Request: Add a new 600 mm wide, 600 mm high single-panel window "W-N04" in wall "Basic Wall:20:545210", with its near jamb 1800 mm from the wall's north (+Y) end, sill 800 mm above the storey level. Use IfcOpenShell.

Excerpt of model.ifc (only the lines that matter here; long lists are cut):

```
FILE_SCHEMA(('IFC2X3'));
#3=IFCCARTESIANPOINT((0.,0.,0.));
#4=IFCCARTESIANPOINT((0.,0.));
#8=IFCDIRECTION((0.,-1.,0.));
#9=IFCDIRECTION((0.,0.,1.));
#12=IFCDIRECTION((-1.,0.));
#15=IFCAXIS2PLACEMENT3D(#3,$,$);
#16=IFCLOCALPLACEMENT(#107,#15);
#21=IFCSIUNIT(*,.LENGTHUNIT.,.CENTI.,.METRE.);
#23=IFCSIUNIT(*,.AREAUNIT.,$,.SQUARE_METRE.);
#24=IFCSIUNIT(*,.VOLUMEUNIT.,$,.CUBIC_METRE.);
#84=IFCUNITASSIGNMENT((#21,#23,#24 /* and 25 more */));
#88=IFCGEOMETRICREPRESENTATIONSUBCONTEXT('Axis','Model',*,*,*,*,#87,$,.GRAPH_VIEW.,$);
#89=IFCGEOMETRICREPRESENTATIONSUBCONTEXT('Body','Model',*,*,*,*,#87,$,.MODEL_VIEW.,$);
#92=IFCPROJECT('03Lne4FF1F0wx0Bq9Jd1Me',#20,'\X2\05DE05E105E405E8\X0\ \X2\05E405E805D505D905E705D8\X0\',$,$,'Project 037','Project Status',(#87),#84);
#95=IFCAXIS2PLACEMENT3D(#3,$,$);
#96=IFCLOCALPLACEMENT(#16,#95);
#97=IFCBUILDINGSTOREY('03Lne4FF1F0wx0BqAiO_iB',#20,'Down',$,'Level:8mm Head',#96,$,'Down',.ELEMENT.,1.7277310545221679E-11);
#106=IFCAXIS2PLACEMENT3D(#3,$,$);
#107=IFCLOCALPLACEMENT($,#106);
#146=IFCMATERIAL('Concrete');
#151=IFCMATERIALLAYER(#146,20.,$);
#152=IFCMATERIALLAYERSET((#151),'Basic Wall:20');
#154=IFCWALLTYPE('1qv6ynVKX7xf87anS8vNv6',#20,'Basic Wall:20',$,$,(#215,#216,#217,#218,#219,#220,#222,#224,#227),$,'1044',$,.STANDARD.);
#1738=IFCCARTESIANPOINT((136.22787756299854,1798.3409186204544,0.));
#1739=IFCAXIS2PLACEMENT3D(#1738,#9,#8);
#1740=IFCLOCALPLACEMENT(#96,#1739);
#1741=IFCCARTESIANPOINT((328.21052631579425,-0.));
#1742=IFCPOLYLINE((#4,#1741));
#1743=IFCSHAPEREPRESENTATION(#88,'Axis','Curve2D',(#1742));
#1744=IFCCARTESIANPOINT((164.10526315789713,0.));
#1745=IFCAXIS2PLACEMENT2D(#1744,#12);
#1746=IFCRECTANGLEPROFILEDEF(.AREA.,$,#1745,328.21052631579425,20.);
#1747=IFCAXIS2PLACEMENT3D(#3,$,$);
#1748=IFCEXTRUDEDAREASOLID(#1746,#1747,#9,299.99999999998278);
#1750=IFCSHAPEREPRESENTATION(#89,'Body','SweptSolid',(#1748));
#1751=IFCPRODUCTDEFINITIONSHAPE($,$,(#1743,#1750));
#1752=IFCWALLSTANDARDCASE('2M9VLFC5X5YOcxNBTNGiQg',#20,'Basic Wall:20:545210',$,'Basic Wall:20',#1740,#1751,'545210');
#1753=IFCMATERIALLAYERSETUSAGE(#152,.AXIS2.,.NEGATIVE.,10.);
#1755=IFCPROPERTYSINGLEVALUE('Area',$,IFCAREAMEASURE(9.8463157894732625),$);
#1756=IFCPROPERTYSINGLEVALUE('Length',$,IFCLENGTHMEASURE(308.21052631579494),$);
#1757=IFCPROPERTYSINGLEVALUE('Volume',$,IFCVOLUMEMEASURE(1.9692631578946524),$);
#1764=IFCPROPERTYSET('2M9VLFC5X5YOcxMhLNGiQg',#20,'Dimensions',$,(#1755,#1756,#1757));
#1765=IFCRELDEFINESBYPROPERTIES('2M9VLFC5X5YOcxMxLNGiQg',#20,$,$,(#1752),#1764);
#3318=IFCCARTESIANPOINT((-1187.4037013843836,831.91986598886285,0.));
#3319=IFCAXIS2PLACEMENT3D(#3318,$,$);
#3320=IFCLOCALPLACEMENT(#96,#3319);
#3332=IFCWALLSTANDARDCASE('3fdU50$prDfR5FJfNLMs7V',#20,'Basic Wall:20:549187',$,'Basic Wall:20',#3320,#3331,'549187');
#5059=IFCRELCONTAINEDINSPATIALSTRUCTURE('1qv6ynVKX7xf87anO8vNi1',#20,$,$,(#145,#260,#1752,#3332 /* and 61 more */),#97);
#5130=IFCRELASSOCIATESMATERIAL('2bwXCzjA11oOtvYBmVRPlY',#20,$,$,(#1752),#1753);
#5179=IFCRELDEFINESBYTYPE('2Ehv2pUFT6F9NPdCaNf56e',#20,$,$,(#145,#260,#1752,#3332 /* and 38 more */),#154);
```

```python
import numpy as np
import ifcopenshell
import ifcopenshell.api.feature
import ifcopenshell.api.geometry
import ifcopenshell.api.pset
import ifcopenshell.api.root
import ifcopenshell.api.spatial
import ifcopenshell.api.type
import ifcopenshell.geom
import ifcopenshell.util.element
import ifcopenshell.util.placement
import ifcopenshell.util.representation
import ifcopenshell.util.shape
import ifcopenshell.util.unit

model = ifcopenshell.open("model.ifc")
unit_scale = ifcopenshell.util.unit.calculate_unit_scale(model)
area_scale = ifcopenshell.util.unit.calculate_unit_scale(model, "AREAUNIT")
volume_scale = ifcopenshell.util.unit.calculate_unit_scale(model, "VOLUMEUNIT")
settings = ifcopenshell.geom.settings()


def volume(element):
    """Net volume in cubic metres, openings subtracted."""
    shape = ifcopenshell.geom.create_shape(settings, element)
    return ifcopenshell.util.shape.get_volume(shape.geometry)


wall = model.by_guid("2M9VLFC5X5YOcxNBTNGiQg")
storey = ifcopenshell.util.element.get_container(wall, ifc_class="IfcBuildingStorey")
context = ifcopenshell.util.representation.get_context(model, "Model", "Body", "MODEL_VIEW")
before = volume(wall)

width, height, from_end, sill = 0.6, 0.6, 1.8, 0.8  # metres

# The wall runs along its own X axis, and the end named is its -X end.
wall_shape = ifcopenshell.geom.create_shape(settings, wall)
x, y, z = ifcopenshell.util.shape.get_vertices(wall_shape.geometry).T
start = x.min() + from_end
face, thickness = float(y.min()), float(y.max() - y.min())
wall_matrix = ifcopenshell.util.placement.get_local_placement(wall.ObjectPlacement)
level = ifcopenshell.util.placement.get_local_placement(storey.ObjectPlacement)[2, 3]


def in_wall(x, y):
    """Placement at x, y metres in the wall's axes, at sill height."""
    matrix = wall_matrix.copy()
    matrix[:, 3] = wall_matrix @ np.array([x / unit_scale, y / unit_scale, 0.0, 1.0])
    matrix[2, 3] = level + sill / unit_scale
    return matrix


# Opening: a box that overshoots both wall faces by 50 mm.
opening = ifcopenshell.api.root.create_entity(model, ifc_class="IfcOpeningElement")
box = ifcopenshell.api.geometry.add_wall_representation(
    model, context=context, length=width, height=height, thickness=thickness + 0.1
)
ifcopenshell.api.geometry.assign_representation(model, product=opening, representation=box)
ifcopenshell.api.geometry.edit_object_placement(model, product=opening, matrix=in_wall(start, face - 0.05), is_si=False)
ifcopenshell.api.feature.add_feature(model, feature=opening, element=wall)

window = ifcopenshell.api.root.create_entity(model, ifc_class="IfcWindow", name="W-N04")
window.OverallWidth, window.OverallHeight = width / unit_scale, height / unit_scale
body = ifcopenshell.api.geometry.add_window_representation(
    model,
    context=context,
    overall_width=window.OverallWidth,
    overall_height=window.OverallHeight,
    partition_type="SINGLE_PANEL",
)
ifcopenshell.api.geometry.assign_representation(model, product=window, representation=body)
ifcopenshell.api.spatial.assign_container(model, products=[window], relating_structure=storey)
fills = ifcopenshell.api.feature.add_filling(model, opening=opening, element=window)
fills.OwnerHistory = window.OwnerHistory  # required in IFC2X3

# IFC2X3 keeps the operation on the window style.
style = ifcopenshell.api.root.create_entity(model, ifc_class="IfcWindowStyle", name="W-N04")
style.OperationType, style.ConstructionType = "SINGLE_PANEL", "NOTDEFINED"
style.ParameterTakesPrecedence = style.Sizeable = False
ifcopenshell.api.type.assign_type(model, related_objects=[window], relating_type=style)

# Centre the window in the wall's thickness.
ifcopenshell.api.geometry.edit_object_placement(model, product=window, matrix=in_wall(start, face), is_si=False)
window_shape = ifcopenshell.geom.create_shape(settings, window)
depth = ifcopenshell.util.shape.get_vertices(window_shape.geometry)[:, 1]
offset = face + thickness / 2 - (depth.min() + depth.max()) / 2
ifcopenshell.api.geometry.edit_object_placement(model, product=window, matrix=in_wall(start, offset), is_si=False)

after = volume(wall)

# Update the wall's stored quantities.
pset = model.by_id(ifcopenshell.util.element.get_pset(wall, "Dimensions", should_inherit=False)["id"])
ifcopenshell.api.pset.edit_pset(model, pset=pset, properties={
    "Area": model.create_entity("IfcAreaMeasure", after / thickness / area_scale),
    "Volume": model.create_entity("IfcVolumeMeasure", after / volume_scale),
})

print(f"wall volume {before:.3f} -> {after:.3f} m3")

model.write("model-out.ifc")
```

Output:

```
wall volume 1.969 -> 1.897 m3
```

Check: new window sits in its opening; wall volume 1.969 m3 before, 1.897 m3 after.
